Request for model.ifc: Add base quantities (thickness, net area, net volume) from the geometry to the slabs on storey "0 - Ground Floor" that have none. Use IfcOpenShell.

First a look at what the model holds.

```python
import ifcopenshell
import ifcopenshell.util.element
import ifcopenshell.util.unit

model = ifcopenshell.open("model.ifc")
print(model.schema)
for unit_type in ("LENGTHUNIT", "AREAUNIT", "VOLUMEUNIT"):
    print(unit_type, ifcopenshell.util.unit.calculate_unit_scale(model, unit_type))
storey = next(s for s in model.by_type("IfcBuildingStorey") if s.Name == "0 - Ground Floor")
slabs = [e for e in ifcopenshell.util.element.get_decomposition(storey) if e.is_a("IfcSlab")]
for e in sorted(slabs, key=lambda e: e.id()):
    print(e.id(), e.is_a(), e.Name, list(ifcopenshell.util.element.get_psets(e, qtos_only=True)), sep=" | ")
```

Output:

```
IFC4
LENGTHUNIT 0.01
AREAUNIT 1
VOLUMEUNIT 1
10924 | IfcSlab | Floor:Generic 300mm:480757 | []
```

```python
import ifcopenshell
import ifcopenshell.api.pset
import ifcopenshell.geom
import ifcopenshell.util.element
import ifcopenshell.util.shape
import ifcopenshell.util.unit

model = ifcopenshell.open("model.ifc")
unit_scale = ifcopenshell.util.unit.calculate_unit_scale(model)
area_scale = ifcopenshell.util.unit.calculate_unit_scale(model, "AREAUNIT")
volume_scale = ifcopenshell.util.unit.calculate_unit_scale(model, "VOLUMEUNIT")
settings = ifcopenshell.geom.settings()

storey = next(s for s in model.by_type("IfcBuildingStorey") if s.Name == "0 - Ground Floor")
slabs = [e for e in ifcopenshell.util.element.get_decomposition(storey) if e.is_a("IfcSlab")]

for e in sorted(slabs, key=lambda e: e.id()):
    if ifcopenshell.util.element.get_psets(e, qtos_only=True, should_inherit=False):
        continue
    # Geometry comes back in metres, in the element's own axes.
    shape = ifcopenshell.geom.create_shape(settings, e)
    values = {
        "Width": ifcopenshell.util.shape.get_z(shape.geometry) / unit_scale,
        "NetArea": ifcopenshell.util.shape.get_footprint_area(shape.geometry) / area_scale,
        "NetVolume": ifcopenshell.util.shape.get_volume(shape.geometry) / volume_scale,
    }
    qto = ifcopenshell.api.pset.add_qto(model, product=e, name="Qto_SlabBaseQuantities")
    ifcopenshell.api.pset.edit_qto(model, qto=qto, properties=values)
    print(e.id(), {k: round(v, 3) for k, v in values.items()})

model.write("model_v2.ifc")
```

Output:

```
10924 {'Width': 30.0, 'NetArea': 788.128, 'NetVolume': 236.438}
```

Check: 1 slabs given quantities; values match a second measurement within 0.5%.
